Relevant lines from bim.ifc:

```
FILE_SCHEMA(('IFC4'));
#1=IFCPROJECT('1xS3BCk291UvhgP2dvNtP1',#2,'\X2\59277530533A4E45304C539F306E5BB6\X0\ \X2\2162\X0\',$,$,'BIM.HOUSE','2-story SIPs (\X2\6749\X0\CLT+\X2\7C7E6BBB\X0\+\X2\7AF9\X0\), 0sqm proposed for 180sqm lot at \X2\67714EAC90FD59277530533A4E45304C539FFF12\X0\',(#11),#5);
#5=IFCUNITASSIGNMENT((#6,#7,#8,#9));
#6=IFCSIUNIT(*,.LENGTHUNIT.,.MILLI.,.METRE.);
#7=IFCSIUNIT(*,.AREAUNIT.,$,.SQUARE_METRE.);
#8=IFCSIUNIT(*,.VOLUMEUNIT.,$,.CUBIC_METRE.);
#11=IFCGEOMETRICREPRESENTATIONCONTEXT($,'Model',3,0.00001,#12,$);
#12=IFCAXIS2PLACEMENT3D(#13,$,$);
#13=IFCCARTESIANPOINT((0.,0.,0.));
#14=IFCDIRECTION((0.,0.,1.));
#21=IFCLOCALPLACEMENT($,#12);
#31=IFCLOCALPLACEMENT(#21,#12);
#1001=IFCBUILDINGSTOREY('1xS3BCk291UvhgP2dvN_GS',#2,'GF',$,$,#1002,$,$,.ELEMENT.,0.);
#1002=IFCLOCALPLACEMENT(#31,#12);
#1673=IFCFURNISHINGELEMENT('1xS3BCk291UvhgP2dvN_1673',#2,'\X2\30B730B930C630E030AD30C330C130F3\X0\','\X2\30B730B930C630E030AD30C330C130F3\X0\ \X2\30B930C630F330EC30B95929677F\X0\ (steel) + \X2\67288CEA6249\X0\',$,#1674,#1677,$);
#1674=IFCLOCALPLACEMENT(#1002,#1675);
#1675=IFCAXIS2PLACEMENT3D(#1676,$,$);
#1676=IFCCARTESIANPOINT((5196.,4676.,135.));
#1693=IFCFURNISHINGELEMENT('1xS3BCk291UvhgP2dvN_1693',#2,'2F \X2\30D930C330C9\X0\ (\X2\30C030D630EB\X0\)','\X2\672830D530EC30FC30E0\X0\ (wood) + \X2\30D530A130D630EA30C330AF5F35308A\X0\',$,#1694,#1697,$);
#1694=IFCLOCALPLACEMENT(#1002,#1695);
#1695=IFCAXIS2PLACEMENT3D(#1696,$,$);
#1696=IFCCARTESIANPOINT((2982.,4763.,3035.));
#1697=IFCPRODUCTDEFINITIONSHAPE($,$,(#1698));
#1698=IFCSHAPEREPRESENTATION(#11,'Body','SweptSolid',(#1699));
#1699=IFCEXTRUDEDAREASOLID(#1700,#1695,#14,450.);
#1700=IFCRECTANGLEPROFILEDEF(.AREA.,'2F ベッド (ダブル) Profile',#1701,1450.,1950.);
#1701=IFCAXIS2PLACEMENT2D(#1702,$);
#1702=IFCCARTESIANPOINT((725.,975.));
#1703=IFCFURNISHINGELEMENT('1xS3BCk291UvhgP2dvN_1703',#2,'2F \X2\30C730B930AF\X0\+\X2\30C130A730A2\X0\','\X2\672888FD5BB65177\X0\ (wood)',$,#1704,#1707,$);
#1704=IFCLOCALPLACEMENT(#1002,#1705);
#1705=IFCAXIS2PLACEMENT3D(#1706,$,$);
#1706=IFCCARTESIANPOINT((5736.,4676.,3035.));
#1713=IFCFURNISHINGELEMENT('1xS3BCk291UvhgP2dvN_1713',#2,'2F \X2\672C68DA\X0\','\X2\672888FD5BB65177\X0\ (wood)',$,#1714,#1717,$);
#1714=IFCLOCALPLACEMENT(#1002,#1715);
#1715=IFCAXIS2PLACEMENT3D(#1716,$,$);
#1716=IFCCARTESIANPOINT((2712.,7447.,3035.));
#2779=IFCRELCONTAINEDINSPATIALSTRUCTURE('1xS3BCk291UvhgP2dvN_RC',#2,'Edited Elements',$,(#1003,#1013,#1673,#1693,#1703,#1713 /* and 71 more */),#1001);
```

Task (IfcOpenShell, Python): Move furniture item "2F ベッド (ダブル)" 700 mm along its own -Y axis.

```python
import ifcopenshell
import ifcopenshell.api.geometry
import ifcopenshell.util.placement
import ifcopenshell.util.unit

model = ifcopenshell.open("bim.ifc")
unit_scale = ifcopenshell.util.unit.calculate_unit_scale(model)

item = model.by_guid("1xS3BCk291UvhgP2dvN_1693")
matrix = ifcopenshell.util.placement.get_local_placement(item.ObjectPlacement)
matrix[:3, 3] -= matrix[:3, 1] * 0.7 / unit_scale
ifcopenshell.api.geometry.edit_object_placement(model, product=item, matrix=matrix, is_si=False)

print(ifcopenshell.util.placement.get_local_placement(item.ObjectPlacement).round(3) + 0.0)

model.write("bim_v2.ifc")
```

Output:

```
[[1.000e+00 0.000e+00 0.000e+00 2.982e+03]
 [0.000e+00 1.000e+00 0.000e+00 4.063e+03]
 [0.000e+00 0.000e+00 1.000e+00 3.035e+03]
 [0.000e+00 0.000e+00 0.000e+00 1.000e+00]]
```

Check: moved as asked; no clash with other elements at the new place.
